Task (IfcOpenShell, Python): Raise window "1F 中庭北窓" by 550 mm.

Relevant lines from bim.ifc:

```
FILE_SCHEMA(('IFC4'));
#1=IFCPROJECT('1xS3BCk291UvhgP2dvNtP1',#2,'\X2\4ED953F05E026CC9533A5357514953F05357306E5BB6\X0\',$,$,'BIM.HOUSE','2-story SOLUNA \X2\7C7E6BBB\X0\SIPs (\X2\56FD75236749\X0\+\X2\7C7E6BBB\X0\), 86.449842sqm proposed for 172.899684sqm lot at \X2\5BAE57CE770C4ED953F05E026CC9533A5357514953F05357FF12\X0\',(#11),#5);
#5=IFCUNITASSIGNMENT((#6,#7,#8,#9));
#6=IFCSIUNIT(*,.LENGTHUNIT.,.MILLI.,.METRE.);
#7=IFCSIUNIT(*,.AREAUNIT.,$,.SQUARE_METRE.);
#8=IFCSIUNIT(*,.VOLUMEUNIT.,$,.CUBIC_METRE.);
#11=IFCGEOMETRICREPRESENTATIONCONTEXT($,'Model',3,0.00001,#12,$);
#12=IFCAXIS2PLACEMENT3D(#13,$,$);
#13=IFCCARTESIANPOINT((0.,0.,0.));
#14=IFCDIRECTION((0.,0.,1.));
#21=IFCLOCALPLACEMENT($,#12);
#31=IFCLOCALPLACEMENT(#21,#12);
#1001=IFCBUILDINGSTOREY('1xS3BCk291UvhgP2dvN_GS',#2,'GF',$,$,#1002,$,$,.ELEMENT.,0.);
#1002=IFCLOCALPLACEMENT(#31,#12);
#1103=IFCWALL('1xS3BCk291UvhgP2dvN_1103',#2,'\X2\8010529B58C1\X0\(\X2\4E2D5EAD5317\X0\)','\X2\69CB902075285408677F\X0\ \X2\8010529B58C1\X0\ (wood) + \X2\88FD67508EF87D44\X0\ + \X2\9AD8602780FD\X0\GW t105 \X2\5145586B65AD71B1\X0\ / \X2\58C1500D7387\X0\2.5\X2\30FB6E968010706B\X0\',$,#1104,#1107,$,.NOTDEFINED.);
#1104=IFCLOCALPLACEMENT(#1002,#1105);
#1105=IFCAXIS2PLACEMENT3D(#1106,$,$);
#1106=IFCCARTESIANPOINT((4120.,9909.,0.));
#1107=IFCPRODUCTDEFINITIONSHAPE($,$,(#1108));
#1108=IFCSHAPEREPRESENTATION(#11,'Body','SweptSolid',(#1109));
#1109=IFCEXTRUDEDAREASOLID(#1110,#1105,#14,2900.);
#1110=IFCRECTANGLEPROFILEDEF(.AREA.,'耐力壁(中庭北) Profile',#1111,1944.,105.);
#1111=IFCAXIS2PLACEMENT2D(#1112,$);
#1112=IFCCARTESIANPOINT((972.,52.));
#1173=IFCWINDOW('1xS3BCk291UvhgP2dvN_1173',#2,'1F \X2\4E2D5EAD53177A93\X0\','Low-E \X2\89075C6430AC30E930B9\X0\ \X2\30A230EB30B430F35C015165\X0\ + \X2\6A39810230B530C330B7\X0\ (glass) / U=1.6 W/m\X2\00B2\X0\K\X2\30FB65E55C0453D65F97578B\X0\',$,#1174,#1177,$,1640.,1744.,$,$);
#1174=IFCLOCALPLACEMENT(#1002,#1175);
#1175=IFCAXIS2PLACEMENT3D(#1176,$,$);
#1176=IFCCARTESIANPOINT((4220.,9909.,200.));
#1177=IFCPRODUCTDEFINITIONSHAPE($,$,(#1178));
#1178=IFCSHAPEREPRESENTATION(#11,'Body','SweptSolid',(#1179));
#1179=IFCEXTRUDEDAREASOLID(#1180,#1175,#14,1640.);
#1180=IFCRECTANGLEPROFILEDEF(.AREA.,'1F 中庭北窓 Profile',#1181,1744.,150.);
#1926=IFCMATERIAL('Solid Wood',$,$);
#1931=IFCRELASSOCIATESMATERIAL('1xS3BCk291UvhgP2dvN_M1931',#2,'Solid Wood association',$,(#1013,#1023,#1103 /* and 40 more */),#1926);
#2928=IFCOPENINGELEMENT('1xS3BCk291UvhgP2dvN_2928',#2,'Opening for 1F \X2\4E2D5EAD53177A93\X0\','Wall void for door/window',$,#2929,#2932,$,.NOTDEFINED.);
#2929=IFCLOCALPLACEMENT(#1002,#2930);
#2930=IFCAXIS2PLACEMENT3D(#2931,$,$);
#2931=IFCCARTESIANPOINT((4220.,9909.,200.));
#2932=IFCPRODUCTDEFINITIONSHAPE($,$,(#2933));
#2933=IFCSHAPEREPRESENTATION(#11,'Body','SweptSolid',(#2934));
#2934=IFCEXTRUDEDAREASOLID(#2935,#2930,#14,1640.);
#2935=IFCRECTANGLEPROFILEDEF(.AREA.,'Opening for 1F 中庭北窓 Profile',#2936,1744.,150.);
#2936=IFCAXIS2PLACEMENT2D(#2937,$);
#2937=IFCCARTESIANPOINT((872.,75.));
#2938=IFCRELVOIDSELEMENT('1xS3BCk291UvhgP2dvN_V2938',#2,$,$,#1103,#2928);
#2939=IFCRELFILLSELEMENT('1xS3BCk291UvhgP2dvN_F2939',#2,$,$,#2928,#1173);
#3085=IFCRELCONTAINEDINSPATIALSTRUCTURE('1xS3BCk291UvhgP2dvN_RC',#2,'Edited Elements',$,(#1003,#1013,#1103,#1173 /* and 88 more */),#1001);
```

```python
import numpy as np
import ifcopenshell
import ifcopenshell.api.geometry
import ifcopenshell.util.placement
import ifcopenshell.util.unit

model = ifcopenshell.open("bim.ifc")
unit_scale = ifcopenshell.util.unit.calculate_unit_scale(model)

window = model.by_id(1173)
opening = window.FillsVoids[0].RelatingOpeningElement
dz = 550.0

shift = np.array([0.0, 0.0, dz])
# The window is not placed relative to its opening, so move both.
for product in (opening, window):
    matrix = ifcopenshell.util.placement.get_local_placement(product.ObjectPlacement)
    matrix[:3, 3] += shift
    ifcopenshell.api.geometry.edit_object_placement(model, product=product, matrix=matrix, is_si=False)

print(f"moved by {dz * unit_scale:+.3f} m")

model.write("bim_updated.ifc")
```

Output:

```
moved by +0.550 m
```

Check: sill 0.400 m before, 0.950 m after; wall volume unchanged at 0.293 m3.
